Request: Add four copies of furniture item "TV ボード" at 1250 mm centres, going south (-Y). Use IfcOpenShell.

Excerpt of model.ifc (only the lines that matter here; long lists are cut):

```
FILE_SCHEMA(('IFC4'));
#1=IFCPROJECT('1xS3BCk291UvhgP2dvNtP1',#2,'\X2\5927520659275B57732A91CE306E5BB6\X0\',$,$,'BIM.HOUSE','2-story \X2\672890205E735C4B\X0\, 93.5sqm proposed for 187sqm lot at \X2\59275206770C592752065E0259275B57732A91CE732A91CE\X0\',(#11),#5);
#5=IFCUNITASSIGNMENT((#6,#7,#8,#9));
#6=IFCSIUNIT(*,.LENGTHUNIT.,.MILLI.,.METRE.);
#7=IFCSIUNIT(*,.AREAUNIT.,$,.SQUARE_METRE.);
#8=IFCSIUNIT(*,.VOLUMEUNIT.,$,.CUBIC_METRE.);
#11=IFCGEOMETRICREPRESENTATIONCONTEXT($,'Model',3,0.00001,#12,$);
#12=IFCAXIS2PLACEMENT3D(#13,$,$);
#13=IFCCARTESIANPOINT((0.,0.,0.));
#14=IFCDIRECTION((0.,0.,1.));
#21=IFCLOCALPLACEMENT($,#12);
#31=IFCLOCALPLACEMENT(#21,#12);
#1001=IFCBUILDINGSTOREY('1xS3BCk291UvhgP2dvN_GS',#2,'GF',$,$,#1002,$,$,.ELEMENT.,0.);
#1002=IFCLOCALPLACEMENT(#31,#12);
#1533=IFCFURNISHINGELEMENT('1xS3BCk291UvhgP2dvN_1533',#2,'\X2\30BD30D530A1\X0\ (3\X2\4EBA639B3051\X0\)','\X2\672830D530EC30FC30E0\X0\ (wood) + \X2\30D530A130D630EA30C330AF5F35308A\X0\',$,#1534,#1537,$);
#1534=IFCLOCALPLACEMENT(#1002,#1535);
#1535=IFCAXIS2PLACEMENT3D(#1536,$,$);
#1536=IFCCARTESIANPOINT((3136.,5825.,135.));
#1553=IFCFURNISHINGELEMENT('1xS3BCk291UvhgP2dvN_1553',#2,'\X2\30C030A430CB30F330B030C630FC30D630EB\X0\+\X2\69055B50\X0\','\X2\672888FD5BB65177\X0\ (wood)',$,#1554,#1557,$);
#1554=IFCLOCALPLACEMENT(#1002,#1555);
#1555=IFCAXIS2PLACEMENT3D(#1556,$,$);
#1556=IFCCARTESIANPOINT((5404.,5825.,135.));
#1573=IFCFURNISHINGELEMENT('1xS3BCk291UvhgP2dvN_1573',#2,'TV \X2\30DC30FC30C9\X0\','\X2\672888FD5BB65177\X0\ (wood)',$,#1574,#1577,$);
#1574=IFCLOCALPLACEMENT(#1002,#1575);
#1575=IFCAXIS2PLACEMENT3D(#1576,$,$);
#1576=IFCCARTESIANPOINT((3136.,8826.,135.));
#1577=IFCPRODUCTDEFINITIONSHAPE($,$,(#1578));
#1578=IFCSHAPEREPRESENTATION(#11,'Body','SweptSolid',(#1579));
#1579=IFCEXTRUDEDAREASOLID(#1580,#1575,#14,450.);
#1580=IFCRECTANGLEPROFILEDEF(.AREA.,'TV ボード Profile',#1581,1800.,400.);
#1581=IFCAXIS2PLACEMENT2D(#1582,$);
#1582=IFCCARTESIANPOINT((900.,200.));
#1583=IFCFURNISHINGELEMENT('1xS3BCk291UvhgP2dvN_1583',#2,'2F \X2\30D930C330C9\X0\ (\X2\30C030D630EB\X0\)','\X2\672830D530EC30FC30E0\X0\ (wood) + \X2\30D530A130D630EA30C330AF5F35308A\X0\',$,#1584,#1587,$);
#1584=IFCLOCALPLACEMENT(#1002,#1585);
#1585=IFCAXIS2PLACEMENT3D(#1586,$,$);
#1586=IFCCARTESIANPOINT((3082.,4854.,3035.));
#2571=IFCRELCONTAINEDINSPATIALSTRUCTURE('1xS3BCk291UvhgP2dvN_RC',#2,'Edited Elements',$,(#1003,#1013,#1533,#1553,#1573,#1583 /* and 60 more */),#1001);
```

```python
import numpy as np
import ifcopenshell
import ifcopenshell.api.geometry
import ifcopenshell.api.root
import ifcopenshell.util.element
import ifcopenshell.util.placement
import ifcopenshell.util.unit

model = ifcopenshell.open("model.ifc")
unit_scale = ifcopenshell.util.unit.calculate_unit_scale(model)


def reuse_history(source, copy):
    """copy_class also copies each property set's owner history, people and application; keep the originals."""
    for rel in copy.IsDefinedBy:
        if rel.is_a("IfcRelDefinesByProperties") and (history := rel.RelatingPropertyDefinition.OwnerHistory):
            rel.RelatingPropertyDefinition.OwnerHistory = source.OwnerHistory
            ifcopenshell.util.element.remove_deep2(model, history)


source = model.by_guid("1xS3BCk291UvhgP2dvN_1573")
base = ifcopenshell.util.placement.get_local_placement(source.ObjectPlacement)
step = np.array([0.0, -1.0, 0.0]) * 1.25 / unit_scale

for i in range(1, 5):
    copy = ifcopenshell.api.root.copy_class(model, product=source)
    copy.Representation = ifcopenshell.util.element.copy_deep(
        model, source.Representation, exclude=["IfcGeometricRepresentationContext", "IfcRepresentationMap"]
    )
    reuse_history(source, copy)
    matrix = base.copy()
    matrix[:3, 3] += i * step
    print("added at", matrix[:3, 3].round(3) + 0.0)
    ifcopenshell.api.geometry.edit_object_placement(model, product=copy, matrix=matrix, is_si=False)

model.write("model_v2.ifc")
```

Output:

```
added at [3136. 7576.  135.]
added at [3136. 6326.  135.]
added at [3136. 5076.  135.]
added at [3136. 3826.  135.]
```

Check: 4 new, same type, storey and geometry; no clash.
